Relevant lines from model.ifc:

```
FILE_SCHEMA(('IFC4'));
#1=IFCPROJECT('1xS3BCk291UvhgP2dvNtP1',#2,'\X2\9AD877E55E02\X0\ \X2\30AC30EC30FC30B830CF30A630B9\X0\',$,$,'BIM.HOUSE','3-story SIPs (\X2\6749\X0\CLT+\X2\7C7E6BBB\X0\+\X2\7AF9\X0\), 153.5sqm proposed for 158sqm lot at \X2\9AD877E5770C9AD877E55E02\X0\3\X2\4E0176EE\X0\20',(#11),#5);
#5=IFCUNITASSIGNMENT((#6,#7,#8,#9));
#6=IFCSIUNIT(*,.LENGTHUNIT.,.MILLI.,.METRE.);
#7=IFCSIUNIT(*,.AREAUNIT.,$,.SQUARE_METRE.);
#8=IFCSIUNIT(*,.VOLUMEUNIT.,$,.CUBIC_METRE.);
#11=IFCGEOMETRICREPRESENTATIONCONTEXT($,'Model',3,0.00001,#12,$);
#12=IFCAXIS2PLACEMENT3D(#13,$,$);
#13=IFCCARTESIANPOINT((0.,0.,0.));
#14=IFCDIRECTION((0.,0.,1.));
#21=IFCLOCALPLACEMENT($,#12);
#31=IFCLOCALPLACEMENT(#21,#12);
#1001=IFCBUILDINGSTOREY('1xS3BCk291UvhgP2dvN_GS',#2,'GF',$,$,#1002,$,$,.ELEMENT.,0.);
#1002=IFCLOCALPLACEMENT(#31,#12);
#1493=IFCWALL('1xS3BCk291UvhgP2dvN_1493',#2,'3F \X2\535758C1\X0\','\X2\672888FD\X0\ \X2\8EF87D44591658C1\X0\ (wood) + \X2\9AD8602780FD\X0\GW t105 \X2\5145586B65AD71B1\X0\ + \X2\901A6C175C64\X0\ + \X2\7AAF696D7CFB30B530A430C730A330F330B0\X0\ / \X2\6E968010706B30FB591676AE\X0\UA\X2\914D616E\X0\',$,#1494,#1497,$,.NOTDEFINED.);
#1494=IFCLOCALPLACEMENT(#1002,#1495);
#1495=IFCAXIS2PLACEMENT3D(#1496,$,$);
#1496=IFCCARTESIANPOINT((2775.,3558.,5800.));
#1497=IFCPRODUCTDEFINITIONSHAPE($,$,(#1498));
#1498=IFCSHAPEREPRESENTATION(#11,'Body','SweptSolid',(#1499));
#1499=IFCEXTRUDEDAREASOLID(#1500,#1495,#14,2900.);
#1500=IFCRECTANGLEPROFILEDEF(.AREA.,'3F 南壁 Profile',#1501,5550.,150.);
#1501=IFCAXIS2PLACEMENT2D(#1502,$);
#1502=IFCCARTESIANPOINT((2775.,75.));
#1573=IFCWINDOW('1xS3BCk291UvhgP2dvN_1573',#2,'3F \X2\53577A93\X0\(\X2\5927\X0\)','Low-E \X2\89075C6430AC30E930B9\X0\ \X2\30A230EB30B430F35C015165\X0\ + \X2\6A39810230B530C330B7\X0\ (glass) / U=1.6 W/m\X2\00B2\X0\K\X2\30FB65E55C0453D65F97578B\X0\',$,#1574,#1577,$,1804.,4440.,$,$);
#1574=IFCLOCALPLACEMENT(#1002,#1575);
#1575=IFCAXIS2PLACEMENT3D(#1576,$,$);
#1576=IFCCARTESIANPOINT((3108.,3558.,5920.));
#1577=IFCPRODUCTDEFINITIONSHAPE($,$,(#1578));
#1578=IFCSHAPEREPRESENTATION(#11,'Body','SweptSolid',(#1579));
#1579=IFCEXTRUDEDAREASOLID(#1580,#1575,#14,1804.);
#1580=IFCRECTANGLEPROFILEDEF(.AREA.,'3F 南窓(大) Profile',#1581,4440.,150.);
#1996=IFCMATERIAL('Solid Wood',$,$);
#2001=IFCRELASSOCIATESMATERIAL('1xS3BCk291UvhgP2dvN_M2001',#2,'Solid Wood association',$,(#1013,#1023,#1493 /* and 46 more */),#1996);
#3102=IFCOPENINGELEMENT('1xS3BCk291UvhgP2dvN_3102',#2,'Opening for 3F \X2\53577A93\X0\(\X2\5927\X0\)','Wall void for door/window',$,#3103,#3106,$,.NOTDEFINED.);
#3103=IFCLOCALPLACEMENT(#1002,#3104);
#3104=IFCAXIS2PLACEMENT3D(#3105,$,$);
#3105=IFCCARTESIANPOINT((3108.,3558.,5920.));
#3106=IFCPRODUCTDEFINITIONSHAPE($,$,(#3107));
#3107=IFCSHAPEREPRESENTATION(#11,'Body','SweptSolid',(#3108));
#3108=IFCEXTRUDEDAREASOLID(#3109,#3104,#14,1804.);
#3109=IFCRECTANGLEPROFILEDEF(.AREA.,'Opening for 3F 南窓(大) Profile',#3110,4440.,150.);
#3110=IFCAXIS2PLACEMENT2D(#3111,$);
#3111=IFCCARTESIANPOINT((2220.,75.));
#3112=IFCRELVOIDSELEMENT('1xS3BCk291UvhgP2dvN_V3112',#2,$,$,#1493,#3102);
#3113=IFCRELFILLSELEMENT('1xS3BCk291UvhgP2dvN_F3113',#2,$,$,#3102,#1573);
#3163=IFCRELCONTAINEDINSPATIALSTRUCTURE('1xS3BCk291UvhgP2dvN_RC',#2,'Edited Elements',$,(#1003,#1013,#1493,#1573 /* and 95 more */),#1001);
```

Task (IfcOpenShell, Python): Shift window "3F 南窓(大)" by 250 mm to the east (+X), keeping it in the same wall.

```python
import ifcopenshell
import ifcopenshell.api.geometry
import ifcopenshell.util.placement

model = ifcopenshell.open("model.ifc")

window = model.by_guid("1xS3BCk291UvhgP2dvN_1573")
opening = window.FillsVoids[0].RelatingOpeningElement
wall = opening.VoidsElements[0].RelatingBuildingElement

wall_matrix = ifcopenshell.util.placement.get_local_placement(wall.ObjectPlacement)
shift = wall_matrix[:3, 0] * 250.0
before = ifcopenshell.util.placement.get_local_placement(window.ObjectPlacement)[:3, 3].copy()

# The window is not placed relative to its opening, so move both.
for product in (opening, window):
    matrix = ifcopenshell.util.placement.get_local_placement(product.ObjectPlacement)
    matrix[:3, 3] += shift
    ifcopenshell.api.geometry.edit_object_placement(model, product=product, matrix=matrix, is_si=False)

after = ifcopenshell.util.placement.get_local_placement(window.ObjectPlacement)[:3, 3]
print("window moved by", (after - before).round(3) + 0.0)

model.write("model-out.ifc")
```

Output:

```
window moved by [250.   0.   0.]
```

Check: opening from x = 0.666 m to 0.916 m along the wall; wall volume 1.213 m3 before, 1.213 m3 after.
